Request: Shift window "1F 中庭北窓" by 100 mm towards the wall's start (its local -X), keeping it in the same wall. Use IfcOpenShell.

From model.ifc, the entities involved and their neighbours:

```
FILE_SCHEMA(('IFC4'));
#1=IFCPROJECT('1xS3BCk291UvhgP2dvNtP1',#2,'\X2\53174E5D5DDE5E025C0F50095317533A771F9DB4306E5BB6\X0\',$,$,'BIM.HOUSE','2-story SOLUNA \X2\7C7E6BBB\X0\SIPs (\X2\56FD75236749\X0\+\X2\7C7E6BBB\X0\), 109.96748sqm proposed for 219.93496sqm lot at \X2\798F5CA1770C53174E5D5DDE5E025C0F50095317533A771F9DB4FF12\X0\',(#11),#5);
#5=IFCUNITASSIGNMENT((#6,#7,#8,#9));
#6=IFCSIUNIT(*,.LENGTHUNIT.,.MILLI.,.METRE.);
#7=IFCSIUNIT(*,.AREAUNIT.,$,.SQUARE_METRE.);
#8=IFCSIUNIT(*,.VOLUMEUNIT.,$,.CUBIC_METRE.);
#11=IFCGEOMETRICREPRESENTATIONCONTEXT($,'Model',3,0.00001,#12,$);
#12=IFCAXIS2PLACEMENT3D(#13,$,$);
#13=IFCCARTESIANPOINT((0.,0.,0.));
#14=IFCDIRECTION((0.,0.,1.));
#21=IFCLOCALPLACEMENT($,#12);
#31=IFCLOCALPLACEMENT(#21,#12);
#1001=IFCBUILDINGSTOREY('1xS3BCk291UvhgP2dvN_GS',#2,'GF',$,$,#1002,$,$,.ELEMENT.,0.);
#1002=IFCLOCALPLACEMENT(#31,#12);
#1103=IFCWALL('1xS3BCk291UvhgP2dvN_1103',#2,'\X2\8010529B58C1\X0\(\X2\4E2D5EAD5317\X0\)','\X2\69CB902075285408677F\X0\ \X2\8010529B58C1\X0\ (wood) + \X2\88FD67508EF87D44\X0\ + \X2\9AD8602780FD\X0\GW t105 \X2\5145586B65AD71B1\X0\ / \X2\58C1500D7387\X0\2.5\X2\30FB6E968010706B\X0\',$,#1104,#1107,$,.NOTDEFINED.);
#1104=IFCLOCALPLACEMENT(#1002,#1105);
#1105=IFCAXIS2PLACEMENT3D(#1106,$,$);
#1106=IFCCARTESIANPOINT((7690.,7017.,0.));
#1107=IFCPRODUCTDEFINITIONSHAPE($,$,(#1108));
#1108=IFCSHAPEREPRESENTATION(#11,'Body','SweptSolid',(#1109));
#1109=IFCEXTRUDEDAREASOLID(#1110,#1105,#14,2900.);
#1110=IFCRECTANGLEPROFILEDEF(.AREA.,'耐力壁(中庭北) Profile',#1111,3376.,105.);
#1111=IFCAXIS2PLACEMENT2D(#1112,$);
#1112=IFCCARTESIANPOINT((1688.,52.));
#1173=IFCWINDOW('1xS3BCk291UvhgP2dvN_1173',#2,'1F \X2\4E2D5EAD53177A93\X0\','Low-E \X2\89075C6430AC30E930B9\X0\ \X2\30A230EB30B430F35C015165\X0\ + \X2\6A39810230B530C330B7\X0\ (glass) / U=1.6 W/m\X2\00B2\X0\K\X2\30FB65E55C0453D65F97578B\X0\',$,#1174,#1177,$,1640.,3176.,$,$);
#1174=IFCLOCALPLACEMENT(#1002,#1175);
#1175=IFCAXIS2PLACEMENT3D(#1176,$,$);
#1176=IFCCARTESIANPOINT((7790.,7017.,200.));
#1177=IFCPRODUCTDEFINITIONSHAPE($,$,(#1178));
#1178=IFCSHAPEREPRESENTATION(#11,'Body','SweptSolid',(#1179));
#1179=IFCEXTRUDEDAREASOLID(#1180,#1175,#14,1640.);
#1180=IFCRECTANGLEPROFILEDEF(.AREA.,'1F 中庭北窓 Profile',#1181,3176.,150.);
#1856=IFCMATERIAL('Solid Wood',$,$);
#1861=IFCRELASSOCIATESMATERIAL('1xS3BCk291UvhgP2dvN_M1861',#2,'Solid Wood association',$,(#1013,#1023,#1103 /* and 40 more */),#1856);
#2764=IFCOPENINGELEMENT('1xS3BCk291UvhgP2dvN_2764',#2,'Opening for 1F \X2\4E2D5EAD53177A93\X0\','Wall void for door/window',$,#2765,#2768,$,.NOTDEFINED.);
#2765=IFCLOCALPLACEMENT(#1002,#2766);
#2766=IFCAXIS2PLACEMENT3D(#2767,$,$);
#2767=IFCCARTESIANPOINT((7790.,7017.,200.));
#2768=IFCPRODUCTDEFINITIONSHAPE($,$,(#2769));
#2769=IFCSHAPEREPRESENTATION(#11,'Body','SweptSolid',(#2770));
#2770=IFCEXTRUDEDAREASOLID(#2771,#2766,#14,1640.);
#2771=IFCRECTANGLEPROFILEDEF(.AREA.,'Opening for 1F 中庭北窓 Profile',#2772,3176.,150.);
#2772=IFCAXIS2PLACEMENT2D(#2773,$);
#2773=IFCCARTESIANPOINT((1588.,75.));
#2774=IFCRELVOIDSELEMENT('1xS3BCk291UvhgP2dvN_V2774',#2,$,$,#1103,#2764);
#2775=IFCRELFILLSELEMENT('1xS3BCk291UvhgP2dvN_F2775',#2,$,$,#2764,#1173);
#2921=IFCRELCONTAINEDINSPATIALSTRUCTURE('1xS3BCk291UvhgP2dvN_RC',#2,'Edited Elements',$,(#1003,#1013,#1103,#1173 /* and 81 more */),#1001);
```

```python
import ifcopenshell
import ifcopenshell.api.geometry
import ifcopenshell.util.placement
import ifcopenshell.util.unit

model = ifcopenshell.open("model.ifc")
unit_scale = ifcopenshell.util.unit.calculate_unit_scale(model)

window = model.by_id(1173)
opening = window.FillsVoids[0].RelatingOpeningElement
wall = opening.VoidsElements[0].RelatingBuildingElement

wall_matrix = ifcopenshell.util.placement.get_local_placement(wall.ObjectPlacement)
shift = wall_matrix[:3, 0] * -0.1 / unit_scale
before = ifcopenshell.util.placement.get_local_placement(window.ObjectPlacement)[:3, 3].copy()

# The window is not placed relative to its opening, so move both.
for product in (opening, window):
    matrix = ifcopenshell.util.placement.get_local_placement(product.ObjectPlacement)
    matrix[:3, 3] += shift
    ifcopenshell.api.geometry.edit_object_placement(model, product=product, matrix=matrix, is_si=False)

after = ifcopenshell.util.placement.get_local_placement(window.ObjectPlacement)[:3, 3]
print("window moved by", (after - before).round(3) + 0.0)

model.write("model-out.ifc")
```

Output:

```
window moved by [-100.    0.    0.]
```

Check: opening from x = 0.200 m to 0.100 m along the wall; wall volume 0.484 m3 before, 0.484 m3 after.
